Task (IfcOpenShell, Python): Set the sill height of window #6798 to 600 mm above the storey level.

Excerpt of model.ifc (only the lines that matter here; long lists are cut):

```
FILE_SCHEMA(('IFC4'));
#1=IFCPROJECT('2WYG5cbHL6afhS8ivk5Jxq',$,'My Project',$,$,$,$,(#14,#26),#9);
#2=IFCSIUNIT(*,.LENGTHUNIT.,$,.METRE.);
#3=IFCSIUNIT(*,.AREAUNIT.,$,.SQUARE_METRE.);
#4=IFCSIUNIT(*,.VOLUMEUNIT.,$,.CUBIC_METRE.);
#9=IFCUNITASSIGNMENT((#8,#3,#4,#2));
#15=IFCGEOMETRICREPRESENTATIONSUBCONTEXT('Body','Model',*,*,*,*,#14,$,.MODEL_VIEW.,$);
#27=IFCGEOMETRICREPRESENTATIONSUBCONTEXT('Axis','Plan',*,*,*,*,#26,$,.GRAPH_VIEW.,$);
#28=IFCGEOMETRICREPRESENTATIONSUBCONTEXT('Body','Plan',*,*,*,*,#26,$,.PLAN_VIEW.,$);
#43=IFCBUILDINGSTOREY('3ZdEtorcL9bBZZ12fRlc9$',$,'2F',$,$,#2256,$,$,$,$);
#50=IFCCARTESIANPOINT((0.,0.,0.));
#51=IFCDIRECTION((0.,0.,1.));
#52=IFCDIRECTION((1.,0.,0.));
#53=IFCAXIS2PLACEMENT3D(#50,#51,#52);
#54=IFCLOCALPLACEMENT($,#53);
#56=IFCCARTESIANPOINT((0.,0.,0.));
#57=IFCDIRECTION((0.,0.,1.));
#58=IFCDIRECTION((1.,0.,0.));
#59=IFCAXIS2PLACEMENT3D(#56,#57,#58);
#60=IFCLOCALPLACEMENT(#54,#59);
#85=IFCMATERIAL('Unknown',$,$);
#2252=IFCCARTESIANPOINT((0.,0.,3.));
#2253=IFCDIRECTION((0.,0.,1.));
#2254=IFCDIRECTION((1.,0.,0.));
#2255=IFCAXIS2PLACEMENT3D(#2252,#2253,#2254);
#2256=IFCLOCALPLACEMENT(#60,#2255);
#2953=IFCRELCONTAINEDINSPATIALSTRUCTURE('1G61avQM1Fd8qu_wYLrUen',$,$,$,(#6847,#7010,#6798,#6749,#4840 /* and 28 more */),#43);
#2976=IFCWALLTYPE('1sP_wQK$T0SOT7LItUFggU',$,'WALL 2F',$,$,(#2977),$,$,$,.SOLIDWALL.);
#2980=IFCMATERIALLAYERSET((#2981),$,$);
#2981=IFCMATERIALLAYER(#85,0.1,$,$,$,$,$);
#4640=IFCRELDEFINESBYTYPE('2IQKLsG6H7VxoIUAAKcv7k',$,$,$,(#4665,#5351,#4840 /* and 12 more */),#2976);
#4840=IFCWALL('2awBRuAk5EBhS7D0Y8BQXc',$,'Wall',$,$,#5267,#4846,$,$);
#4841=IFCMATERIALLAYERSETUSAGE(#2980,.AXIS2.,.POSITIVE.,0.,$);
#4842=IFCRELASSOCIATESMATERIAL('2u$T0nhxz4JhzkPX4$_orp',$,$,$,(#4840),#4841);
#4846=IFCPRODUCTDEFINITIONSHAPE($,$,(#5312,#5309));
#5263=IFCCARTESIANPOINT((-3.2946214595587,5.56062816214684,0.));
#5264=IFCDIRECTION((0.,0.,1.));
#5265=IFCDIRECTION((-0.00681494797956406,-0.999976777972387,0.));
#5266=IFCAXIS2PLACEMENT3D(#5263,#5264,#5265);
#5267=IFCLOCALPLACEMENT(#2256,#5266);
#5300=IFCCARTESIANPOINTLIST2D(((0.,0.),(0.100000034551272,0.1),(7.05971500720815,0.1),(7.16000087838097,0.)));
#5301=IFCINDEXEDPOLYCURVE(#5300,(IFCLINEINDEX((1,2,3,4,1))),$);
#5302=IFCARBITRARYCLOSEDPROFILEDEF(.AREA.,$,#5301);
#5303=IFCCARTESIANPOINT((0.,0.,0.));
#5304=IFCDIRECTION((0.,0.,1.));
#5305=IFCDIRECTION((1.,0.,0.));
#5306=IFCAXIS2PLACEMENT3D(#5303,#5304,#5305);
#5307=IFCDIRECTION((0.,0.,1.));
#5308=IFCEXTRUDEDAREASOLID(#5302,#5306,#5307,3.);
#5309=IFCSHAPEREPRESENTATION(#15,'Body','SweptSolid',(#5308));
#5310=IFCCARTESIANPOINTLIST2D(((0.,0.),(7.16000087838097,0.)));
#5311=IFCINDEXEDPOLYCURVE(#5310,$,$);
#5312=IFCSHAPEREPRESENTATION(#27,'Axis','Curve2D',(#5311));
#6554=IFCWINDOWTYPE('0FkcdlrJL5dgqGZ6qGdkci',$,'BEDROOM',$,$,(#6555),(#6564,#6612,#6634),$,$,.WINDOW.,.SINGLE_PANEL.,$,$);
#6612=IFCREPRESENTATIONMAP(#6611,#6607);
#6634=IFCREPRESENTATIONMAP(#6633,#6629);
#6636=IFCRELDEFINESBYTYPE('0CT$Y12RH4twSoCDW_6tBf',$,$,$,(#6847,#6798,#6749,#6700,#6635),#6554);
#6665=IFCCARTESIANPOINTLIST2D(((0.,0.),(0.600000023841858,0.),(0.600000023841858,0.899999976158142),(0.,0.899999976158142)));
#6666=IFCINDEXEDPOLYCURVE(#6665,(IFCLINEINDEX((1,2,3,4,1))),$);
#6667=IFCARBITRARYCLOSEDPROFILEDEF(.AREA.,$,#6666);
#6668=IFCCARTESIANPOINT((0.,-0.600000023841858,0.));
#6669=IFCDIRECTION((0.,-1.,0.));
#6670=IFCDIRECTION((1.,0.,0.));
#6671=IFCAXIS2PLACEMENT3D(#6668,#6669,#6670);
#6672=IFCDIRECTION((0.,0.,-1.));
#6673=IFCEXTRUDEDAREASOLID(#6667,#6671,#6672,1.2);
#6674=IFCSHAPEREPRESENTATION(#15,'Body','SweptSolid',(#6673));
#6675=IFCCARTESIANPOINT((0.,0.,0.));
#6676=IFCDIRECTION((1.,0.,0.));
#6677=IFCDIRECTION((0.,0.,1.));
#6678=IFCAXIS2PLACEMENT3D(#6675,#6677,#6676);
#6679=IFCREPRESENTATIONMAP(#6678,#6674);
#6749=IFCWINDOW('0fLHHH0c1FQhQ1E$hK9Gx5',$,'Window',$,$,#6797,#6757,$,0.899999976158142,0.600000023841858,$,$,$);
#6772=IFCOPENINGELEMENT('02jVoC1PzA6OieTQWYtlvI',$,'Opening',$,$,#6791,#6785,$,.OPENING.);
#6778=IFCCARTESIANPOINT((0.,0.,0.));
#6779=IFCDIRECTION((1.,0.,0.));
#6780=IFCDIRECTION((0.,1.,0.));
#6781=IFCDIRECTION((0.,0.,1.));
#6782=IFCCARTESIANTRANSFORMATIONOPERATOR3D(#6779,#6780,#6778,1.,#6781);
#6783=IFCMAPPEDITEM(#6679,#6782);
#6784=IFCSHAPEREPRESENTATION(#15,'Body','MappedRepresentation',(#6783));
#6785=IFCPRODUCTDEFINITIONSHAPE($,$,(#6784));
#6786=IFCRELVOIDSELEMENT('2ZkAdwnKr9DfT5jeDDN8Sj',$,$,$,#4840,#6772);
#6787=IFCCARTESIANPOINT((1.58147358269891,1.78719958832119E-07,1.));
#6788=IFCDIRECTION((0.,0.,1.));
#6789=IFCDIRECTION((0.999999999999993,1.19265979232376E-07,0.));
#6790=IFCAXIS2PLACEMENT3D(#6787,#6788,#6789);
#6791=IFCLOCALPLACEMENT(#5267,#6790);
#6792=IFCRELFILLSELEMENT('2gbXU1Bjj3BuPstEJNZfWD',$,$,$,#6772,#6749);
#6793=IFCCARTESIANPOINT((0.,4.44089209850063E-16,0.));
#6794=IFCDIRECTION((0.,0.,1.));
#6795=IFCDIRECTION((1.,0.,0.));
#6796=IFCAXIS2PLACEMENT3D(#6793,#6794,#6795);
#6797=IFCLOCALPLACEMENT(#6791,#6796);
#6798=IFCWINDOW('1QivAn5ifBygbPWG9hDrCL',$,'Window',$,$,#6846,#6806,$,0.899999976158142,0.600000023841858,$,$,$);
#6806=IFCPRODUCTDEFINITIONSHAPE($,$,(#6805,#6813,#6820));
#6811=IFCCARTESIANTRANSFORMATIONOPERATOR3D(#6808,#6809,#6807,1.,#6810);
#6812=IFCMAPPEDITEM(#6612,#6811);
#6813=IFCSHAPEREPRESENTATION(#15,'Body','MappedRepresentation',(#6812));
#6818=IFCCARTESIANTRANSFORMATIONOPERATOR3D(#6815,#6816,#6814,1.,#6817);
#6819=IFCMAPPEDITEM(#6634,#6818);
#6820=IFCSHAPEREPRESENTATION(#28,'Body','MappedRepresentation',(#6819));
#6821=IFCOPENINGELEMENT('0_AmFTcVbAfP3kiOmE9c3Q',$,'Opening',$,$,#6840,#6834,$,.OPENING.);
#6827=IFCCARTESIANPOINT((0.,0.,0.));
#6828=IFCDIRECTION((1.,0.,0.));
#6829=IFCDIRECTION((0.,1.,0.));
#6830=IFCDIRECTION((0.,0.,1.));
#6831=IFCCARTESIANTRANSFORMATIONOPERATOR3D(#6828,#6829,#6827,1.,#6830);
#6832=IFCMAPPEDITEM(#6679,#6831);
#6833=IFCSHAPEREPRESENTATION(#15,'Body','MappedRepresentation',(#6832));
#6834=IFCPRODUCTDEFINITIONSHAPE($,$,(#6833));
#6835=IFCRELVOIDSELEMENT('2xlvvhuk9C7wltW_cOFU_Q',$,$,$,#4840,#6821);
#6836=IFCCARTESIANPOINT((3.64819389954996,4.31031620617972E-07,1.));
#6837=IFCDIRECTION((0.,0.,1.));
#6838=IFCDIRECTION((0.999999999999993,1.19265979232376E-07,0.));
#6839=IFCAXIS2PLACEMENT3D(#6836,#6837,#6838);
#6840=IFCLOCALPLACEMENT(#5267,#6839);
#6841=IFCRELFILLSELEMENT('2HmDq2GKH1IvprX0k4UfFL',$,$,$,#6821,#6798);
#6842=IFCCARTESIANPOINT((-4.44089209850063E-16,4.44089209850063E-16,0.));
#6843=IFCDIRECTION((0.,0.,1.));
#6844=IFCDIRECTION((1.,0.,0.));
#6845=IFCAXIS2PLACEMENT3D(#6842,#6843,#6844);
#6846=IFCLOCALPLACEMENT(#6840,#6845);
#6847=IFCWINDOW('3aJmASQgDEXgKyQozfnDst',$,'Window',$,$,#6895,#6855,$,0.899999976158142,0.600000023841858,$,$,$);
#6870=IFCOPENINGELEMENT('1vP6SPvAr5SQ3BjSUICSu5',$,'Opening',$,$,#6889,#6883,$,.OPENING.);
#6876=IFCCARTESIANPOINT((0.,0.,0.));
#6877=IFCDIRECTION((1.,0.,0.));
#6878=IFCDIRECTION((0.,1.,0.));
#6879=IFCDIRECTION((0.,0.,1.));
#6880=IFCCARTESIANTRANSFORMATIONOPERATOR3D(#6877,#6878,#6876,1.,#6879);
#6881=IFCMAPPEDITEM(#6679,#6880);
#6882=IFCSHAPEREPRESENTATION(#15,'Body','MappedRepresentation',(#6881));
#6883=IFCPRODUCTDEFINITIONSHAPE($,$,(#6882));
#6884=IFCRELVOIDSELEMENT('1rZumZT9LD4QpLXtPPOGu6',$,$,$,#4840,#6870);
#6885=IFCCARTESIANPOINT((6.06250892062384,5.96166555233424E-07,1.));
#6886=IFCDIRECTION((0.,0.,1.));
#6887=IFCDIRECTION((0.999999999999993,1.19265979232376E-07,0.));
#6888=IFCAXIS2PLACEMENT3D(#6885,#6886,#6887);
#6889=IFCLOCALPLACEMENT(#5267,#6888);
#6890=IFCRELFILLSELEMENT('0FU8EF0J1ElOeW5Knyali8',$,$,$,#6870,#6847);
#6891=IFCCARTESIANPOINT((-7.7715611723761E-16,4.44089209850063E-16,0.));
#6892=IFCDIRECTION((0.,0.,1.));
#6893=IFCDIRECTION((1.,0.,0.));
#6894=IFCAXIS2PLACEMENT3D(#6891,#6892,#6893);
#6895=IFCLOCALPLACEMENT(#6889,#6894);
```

```python
import numpy as np
import ifcopenshell
import ifcopenshell.api.geometry
import ifcopenshell.geom
import ifcopenshell.util.element
import ifcopenshell.util.placement
import ifcopenshell.util.shape
import ifcopenshell.util.unit

model = ifcopenshell.open("model.ifc")
unit_scale = ifcopenshell.util.unit.calculate_unit_scale(model)

window = model.by_id(6798)
opening = window.FillsVoids[0].RelatingOpeningElement
storey = ifcopenshell.util.element.get_container(window, ifc_class="IfcBuildingStorey")
level = ifcopenshell.util.placement.get_local_placement(storey.ObjectPlacement)[2, 3]

# The opening's origin need not be at the sill, so measure its lowest point.
shape = ifcopenshell.geom.create_shape(ifcopenshell.geom.settings(), opening)
bottom = ifcopenshell.util.shape.get_shape_bottom_elevation(shape, shape.geometry) / unit_scale
dz = level + 0.6 / unit_scale - bottom

shift = np.array([0.0, 0.0, dz])
# The window is placed relative to its opening, so it follows when the opening moves.
matrix = ifcopenshell.util.placement.get_local_placement(opening.ObjectPlacement)
matrix[:3, 3] += shift
ifcopenshell.api.geometry.edit_object_placement(
    model, product=opening, matrix=matrix, is_si=False, should_transform_children=True
)

print(f"moved by {dz * unit_scale:+.3f} m")

model.write("model-out.ifc")
```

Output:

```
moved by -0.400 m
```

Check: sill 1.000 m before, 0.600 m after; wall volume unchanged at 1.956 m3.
